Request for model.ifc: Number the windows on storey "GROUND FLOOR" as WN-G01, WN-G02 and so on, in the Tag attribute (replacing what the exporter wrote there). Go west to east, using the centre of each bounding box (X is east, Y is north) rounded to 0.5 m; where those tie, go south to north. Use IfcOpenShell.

First a look at what the model holds.

```python
import ifcopenshell
import ifcopenshell.util.element
import ifcopenshell.util.placement

model = ifcopenshell.open("model.ifc")
print(model.schema)
storey = next(s for s in model.by_type("IfcBuildingStorey") if s.Name == "GROUND FLOOR")
windows = [e for e in ifcopenshell.util.element.get_decomposition(storey) if e.is_a("IfcWindow")]
for e in sorted(windows, key=lambda e: e.id()):
    origin = ifcopenshell.util.placement.get_local_placement(e.ObjectPlacement)[:3, 3]
    print(e.id(), e.Tag, e.Name, origin.round(2) + 0.0, sep=" | ")
```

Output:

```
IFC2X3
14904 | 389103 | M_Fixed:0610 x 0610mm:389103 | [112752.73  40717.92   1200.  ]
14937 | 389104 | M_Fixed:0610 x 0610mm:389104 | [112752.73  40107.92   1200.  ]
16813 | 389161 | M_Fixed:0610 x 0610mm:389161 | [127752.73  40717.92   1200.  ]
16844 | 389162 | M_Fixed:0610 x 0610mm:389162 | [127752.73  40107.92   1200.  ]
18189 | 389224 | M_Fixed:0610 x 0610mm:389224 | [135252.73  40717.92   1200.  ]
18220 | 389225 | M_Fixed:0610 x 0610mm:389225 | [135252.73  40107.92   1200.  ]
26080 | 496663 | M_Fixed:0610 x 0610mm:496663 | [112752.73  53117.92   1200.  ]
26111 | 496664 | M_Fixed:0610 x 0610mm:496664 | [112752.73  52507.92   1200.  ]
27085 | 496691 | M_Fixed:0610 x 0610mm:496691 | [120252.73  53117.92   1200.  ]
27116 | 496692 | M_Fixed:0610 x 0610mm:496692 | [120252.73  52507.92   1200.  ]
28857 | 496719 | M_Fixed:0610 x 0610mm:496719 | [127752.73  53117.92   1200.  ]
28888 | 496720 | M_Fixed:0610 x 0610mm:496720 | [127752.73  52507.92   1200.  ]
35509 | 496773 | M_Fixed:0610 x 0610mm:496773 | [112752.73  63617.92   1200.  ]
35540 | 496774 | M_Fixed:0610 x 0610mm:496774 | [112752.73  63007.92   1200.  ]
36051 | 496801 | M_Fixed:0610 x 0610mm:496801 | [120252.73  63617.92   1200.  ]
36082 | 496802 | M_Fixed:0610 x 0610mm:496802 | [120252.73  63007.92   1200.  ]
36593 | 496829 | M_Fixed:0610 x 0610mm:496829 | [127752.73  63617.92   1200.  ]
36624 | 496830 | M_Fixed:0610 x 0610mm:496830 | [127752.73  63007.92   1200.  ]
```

```python
import ifcopenshell
import ifcopenshell.geom
import ifcopenshell.util.element
import ifcopenshell.util.shape

model = ifcopenshell.open("model.ifc")
settings = ifcopenshell.geom.settings()
settings.set("use-world-coords", True)


def centre(element):
    shape = ifcopenshell.geom.create_shape(settings, element)
    return ifcopenshell.util.shape.get_bbox_centroid(shape.geometry)


storey = next(s for s in model.by_type("IfcBuildingStorey") if s.Name == "GROUND FLOOR")
windows = [e for e in ifcopenshell.util.element.get_decomposition(storey) if e.is_a("IfcWindow")]

# Insertion points can sit at a corner or the storey origin, so sort by the geometry (in metres).
centres = {e: centre(e) for e in windows}
windows.sort(key=lambda e: (round(centres[e][0] / 0.5), centres[e][1]))

for i, e in enumerate(windows, start=1):
    number = f"WN-G{i:02d}"
    e.Tag = number
    print(e.id(), number)

model.write("model_rev.ifc")
```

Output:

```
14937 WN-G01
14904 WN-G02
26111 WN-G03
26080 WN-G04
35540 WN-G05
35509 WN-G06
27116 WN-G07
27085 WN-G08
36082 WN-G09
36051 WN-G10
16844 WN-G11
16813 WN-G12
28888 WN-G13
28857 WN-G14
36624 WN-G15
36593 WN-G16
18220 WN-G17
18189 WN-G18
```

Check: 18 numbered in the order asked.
